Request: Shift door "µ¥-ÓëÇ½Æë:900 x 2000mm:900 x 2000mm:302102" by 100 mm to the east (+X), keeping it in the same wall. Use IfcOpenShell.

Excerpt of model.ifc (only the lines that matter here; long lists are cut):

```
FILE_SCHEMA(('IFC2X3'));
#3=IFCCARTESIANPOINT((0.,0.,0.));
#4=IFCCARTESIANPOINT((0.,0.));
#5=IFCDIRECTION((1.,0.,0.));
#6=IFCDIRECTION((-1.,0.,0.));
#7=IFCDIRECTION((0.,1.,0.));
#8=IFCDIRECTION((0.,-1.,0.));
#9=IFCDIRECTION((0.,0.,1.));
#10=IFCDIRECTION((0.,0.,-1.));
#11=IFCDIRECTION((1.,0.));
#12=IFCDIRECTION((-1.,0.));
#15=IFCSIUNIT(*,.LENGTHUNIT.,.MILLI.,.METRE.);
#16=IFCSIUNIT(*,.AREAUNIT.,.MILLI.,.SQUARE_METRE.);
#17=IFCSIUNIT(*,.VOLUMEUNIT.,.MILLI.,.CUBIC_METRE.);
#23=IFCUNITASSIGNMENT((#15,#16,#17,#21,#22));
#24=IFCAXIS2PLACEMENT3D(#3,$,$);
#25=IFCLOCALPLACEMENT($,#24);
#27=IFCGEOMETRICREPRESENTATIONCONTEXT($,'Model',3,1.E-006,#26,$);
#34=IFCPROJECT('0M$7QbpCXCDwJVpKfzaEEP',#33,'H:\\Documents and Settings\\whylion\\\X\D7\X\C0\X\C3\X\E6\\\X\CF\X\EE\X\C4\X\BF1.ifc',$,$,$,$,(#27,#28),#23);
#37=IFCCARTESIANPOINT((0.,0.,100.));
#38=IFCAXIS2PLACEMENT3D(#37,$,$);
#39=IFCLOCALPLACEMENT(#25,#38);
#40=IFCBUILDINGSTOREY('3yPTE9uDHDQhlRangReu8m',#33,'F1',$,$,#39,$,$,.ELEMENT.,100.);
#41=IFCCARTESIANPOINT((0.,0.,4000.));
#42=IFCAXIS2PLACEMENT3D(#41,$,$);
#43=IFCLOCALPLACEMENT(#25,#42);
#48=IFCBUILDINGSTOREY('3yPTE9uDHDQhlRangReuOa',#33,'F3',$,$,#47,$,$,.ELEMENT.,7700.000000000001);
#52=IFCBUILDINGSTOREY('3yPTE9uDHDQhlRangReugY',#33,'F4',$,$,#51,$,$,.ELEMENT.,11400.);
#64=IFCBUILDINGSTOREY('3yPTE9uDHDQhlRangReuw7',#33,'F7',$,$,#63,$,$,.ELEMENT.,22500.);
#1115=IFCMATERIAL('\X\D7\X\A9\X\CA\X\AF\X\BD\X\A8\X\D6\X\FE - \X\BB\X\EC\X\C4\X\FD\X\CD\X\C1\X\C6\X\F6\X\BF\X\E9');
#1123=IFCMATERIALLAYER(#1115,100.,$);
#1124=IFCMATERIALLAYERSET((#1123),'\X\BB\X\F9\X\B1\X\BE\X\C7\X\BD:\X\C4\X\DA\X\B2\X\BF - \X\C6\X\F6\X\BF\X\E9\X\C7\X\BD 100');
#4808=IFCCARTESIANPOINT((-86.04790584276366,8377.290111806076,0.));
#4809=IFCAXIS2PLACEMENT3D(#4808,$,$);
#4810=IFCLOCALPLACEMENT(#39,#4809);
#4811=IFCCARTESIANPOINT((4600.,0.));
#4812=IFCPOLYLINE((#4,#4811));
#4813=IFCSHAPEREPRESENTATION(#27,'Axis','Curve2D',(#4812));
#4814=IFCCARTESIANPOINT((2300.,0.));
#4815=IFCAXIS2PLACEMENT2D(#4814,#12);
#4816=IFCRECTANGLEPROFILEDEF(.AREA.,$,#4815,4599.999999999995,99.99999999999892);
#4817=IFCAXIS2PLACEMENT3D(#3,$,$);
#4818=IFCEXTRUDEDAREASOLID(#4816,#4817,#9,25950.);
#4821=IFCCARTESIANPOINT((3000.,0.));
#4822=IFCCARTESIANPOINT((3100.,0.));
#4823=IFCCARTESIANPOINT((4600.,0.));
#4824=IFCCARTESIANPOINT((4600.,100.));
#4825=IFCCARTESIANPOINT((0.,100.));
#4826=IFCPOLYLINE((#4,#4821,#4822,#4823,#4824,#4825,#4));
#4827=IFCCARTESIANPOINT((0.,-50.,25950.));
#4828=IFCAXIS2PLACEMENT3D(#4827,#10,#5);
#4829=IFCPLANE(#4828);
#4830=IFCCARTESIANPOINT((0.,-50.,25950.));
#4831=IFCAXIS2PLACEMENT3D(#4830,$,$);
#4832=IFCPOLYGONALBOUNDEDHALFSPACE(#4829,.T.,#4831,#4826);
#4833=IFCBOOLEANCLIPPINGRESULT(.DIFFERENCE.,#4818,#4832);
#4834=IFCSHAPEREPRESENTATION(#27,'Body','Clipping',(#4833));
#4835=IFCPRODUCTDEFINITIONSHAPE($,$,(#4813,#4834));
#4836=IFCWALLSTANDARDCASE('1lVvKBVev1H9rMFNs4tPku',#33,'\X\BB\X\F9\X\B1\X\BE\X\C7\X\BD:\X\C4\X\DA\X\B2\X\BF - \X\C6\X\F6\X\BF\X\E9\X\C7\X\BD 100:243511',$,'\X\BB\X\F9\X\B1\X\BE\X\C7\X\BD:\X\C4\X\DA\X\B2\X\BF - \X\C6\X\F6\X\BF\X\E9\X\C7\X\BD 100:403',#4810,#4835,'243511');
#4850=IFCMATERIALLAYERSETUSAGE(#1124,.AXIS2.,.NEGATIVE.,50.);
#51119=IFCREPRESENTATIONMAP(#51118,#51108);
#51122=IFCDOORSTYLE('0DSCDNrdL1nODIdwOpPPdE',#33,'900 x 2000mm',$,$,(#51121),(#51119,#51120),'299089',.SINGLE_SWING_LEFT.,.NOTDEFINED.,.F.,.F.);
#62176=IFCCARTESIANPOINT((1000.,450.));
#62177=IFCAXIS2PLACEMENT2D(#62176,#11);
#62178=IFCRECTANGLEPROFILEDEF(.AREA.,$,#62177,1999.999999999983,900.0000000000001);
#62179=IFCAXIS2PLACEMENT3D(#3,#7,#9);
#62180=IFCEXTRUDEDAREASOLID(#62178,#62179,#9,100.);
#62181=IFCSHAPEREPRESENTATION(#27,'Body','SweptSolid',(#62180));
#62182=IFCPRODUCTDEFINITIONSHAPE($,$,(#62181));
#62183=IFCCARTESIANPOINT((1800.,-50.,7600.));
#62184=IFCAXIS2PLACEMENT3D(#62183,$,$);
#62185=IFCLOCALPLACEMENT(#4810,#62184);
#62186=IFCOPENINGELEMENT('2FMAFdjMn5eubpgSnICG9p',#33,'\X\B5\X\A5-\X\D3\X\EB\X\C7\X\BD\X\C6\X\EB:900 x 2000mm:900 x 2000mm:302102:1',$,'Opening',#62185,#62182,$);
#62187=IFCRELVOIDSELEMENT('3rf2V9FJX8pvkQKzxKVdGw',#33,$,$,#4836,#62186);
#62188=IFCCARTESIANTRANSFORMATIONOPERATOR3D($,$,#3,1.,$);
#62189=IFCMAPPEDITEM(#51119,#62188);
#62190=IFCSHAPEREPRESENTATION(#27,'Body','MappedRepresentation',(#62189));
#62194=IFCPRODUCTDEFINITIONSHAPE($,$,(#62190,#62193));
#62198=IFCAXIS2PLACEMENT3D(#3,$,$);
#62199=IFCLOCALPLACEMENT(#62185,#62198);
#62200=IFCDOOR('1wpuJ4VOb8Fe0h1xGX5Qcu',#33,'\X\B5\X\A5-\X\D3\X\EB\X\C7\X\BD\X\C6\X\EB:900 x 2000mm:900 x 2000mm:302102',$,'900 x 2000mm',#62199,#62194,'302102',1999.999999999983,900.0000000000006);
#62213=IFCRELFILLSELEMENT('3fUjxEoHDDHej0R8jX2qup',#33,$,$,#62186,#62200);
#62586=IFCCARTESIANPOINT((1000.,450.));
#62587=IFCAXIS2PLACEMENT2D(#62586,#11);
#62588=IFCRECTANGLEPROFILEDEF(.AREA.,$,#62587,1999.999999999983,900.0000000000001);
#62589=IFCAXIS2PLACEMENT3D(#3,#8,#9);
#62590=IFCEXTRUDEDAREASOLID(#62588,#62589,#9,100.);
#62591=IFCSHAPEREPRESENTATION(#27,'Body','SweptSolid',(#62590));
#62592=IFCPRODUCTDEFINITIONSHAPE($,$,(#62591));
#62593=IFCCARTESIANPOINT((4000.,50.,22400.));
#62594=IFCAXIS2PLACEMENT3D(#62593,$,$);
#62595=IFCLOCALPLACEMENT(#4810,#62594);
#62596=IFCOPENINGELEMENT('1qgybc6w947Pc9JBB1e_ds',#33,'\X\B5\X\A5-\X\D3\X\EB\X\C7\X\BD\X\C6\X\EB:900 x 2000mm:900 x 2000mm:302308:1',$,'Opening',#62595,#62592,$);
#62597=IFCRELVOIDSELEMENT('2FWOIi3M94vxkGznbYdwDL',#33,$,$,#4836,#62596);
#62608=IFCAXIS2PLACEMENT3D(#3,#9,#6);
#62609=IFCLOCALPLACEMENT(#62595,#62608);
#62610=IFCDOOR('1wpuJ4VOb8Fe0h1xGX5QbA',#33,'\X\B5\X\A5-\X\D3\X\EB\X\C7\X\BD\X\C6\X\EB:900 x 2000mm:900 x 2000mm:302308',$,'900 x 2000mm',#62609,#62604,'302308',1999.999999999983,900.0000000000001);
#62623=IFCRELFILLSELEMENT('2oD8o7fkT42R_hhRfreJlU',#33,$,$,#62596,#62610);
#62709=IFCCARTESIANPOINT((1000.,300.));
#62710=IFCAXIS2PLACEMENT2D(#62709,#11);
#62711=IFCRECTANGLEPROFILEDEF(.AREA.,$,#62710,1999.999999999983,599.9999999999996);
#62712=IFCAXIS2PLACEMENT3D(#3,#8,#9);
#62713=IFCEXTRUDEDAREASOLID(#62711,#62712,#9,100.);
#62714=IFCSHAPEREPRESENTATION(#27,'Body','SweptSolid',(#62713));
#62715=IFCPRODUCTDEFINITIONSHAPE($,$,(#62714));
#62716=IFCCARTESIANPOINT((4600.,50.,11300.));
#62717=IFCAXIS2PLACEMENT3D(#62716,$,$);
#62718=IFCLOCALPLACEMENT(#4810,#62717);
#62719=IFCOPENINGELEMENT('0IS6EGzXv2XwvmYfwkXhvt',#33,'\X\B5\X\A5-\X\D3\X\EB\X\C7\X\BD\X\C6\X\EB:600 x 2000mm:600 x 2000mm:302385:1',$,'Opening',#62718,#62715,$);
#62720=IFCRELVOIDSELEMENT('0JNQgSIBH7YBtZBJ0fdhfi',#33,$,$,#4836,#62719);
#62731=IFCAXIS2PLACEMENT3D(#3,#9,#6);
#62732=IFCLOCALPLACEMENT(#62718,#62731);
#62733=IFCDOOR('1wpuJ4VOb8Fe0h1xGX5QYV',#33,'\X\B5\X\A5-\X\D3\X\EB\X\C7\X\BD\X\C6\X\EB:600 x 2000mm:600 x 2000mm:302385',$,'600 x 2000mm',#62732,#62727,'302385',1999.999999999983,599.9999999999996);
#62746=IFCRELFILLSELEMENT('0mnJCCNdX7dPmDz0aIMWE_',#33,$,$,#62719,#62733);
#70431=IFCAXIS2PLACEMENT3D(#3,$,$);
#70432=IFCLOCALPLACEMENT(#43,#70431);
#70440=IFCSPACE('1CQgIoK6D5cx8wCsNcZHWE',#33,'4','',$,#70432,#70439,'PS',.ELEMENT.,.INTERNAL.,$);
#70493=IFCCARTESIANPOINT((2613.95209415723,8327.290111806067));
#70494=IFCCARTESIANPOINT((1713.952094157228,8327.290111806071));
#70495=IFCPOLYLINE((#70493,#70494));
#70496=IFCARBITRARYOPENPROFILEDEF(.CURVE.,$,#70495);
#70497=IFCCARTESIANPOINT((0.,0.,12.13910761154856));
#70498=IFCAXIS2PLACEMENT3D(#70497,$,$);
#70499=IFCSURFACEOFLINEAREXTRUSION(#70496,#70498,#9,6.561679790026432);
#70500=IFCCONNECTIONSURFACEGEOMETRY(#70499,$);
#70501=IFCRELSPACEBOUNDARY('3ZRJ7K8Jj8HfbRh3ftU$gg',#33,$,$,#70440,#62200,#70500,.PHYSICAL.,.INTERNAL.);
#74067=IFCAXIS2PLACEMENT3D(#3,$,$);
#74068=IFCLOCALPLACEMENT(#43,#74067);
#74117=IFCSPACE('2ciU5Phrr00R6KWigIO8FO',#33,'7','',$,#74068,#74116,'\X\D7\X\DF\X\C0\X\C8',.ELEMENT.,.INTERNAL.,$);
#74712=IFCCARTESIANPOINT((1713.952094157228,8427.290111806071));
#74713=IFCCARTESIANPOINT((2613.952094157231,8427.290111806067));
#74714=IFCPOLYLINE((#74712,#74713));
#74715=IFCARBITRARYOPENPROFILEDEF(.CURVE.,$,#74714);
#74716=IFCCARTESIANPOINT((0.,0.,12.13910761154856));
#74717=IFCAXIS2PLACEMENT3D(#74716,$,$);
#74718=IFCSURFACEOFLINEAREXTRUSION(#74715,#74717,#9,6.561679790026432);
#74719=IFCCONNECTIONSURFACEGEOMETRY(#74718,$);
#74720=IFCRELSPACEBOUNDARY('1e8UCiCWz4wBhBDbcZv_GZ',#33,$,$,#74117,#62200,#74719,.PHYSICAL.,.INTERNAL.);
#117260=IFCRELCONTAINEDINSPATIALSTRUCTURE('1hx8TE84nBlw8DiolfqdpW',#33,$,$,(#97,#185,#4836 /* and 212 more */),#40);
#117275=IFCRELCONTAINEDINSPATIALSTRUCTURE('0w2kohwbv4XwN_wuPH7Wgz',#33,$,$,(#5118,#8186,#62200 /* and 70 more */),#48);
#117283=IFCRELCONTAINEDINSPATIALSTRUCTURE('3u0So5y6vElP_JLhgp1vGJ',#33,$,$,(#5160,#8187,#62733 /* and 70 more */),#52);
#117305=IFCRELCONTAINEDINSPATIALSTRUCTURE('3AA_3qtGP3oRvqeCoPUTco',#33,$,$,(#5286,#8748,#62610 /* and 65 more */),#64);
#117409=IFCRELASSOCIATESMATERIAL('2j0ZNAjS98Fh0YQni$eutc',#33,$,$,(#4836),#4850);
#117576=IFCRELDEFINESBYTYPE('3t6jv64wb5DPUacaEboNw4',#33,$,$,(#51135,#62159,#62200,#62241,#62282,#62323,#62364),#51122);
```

```python
import numpy as np
import ifcopenshell
import ifcopenshell.api.geometry
import ifcopenshell.util.placement
import ifcopenshell.util.unit

model = ifcopenshell.open("model.ifc")
unit_scale = ifcopenshell.util.unit.calculate_unit_scale(model)

door = model.by_id(62200)
opening = door.FillsVoids[0].RelatingOpeningElement
wall = opening.VoidsElements[0].RelatingBuildingElement

wall_matrix = ifcopenshell.util.placement.get_local_placement(wall.ObjectPlacement)
shift = wall_matrix[:3, 0] * 0.1 / unit_scale
before = ifcopenshell.util.placement.get_local_placement(door.ObjectPlacement)[:3, 3].copy()

# The door is placed relative to its opening, so it follows when the opening moves.
matrix = ifcopenshell.util.placement.get_local_placement(opening.ObjectPlacement)
matrix[:3, 3] += shift
ifcopenshell.api.geometry.edit_object_placement(
    model, product=opening, matrix=matrix, is_si=False, should_transform_children=True
)

# Space boundary surfaces are stored in each space's coordinates; move them too.
for rel in door.ProvidesBoundaries:
    if not rel.ConnectionGeometry:
        continue
    surface = rel.ConnectionGeometry.SurfaceOnRelatingElement
    space_matrix = ifcopenshell.util.placement.get_local_placement(rel.RelatingSpace.ObjectPlacement)
    point = np.array(surface.Position.Location.Coordinates) + space_matrix[:3, :3].T @ shift
    surface.Position = model.createIfcAxis2Placement3D(
        model.createIfcCartesianPoint(point.tolist()), surface.Position.Axis, surface.Position.RefDirection
    )

after = ifcopenshell.util.placement.get_local_placement(door.ObjectPlacement)[:3, 3]
print("door moved by", (after - before).round(3) + 0.0)

model.write("model_v2.ifc")
```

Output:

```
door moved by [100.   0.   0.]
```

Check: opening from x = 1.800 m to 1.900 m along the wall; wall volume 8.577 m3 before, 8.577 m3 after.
